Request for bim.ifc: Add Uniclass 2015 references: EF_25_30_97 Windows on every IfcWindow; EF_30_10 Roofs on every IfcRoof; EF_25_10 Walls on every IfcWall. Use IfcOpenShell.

First a look at what the model holds.

```python
import ifcopenshell

model = ifcopenshell.open("bim.ifc")
print(model.schema)
print("classifications:", [c.Name for c in model.by_type("IfcClassification")])
for ifc_class in ("IfcDoor", "IfcRoof", "IfcStair", "IfcWall", "IfcWindow"):
    print(ifc_class, len(model.by_type(ifc_class)))
```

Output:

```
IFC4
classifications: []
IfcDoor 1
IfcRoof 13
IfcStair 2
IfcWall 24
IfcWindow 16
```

```python
import ifcopenshell
import ifcopenshell.api.classification

model = ifcopenshell.open("bim.ifc")

system = ifcopenshell.api.classification.add_classification(model, classification="Uniclass 2015")

codes = {
    "IfcWindow": ("EF_25_30_97", "Windows"),
    "IfcRoof": ("EF_30_10", "Roofs"),
    "IfcWall": ("EF_25_10", "Walls"),
}
for ifc_class, (code, name) in codes.items():
    products = model.by_type(ifc_class)
    ifcopenshell.api.classification.add_reference(
        model, products=products, classification=system, identification=code, name=name
    )
    print(code, len(products))

model.write("bim-out.ifc")
```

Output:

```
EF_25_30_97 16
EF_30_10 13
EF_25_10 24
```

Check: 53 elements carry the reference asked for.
